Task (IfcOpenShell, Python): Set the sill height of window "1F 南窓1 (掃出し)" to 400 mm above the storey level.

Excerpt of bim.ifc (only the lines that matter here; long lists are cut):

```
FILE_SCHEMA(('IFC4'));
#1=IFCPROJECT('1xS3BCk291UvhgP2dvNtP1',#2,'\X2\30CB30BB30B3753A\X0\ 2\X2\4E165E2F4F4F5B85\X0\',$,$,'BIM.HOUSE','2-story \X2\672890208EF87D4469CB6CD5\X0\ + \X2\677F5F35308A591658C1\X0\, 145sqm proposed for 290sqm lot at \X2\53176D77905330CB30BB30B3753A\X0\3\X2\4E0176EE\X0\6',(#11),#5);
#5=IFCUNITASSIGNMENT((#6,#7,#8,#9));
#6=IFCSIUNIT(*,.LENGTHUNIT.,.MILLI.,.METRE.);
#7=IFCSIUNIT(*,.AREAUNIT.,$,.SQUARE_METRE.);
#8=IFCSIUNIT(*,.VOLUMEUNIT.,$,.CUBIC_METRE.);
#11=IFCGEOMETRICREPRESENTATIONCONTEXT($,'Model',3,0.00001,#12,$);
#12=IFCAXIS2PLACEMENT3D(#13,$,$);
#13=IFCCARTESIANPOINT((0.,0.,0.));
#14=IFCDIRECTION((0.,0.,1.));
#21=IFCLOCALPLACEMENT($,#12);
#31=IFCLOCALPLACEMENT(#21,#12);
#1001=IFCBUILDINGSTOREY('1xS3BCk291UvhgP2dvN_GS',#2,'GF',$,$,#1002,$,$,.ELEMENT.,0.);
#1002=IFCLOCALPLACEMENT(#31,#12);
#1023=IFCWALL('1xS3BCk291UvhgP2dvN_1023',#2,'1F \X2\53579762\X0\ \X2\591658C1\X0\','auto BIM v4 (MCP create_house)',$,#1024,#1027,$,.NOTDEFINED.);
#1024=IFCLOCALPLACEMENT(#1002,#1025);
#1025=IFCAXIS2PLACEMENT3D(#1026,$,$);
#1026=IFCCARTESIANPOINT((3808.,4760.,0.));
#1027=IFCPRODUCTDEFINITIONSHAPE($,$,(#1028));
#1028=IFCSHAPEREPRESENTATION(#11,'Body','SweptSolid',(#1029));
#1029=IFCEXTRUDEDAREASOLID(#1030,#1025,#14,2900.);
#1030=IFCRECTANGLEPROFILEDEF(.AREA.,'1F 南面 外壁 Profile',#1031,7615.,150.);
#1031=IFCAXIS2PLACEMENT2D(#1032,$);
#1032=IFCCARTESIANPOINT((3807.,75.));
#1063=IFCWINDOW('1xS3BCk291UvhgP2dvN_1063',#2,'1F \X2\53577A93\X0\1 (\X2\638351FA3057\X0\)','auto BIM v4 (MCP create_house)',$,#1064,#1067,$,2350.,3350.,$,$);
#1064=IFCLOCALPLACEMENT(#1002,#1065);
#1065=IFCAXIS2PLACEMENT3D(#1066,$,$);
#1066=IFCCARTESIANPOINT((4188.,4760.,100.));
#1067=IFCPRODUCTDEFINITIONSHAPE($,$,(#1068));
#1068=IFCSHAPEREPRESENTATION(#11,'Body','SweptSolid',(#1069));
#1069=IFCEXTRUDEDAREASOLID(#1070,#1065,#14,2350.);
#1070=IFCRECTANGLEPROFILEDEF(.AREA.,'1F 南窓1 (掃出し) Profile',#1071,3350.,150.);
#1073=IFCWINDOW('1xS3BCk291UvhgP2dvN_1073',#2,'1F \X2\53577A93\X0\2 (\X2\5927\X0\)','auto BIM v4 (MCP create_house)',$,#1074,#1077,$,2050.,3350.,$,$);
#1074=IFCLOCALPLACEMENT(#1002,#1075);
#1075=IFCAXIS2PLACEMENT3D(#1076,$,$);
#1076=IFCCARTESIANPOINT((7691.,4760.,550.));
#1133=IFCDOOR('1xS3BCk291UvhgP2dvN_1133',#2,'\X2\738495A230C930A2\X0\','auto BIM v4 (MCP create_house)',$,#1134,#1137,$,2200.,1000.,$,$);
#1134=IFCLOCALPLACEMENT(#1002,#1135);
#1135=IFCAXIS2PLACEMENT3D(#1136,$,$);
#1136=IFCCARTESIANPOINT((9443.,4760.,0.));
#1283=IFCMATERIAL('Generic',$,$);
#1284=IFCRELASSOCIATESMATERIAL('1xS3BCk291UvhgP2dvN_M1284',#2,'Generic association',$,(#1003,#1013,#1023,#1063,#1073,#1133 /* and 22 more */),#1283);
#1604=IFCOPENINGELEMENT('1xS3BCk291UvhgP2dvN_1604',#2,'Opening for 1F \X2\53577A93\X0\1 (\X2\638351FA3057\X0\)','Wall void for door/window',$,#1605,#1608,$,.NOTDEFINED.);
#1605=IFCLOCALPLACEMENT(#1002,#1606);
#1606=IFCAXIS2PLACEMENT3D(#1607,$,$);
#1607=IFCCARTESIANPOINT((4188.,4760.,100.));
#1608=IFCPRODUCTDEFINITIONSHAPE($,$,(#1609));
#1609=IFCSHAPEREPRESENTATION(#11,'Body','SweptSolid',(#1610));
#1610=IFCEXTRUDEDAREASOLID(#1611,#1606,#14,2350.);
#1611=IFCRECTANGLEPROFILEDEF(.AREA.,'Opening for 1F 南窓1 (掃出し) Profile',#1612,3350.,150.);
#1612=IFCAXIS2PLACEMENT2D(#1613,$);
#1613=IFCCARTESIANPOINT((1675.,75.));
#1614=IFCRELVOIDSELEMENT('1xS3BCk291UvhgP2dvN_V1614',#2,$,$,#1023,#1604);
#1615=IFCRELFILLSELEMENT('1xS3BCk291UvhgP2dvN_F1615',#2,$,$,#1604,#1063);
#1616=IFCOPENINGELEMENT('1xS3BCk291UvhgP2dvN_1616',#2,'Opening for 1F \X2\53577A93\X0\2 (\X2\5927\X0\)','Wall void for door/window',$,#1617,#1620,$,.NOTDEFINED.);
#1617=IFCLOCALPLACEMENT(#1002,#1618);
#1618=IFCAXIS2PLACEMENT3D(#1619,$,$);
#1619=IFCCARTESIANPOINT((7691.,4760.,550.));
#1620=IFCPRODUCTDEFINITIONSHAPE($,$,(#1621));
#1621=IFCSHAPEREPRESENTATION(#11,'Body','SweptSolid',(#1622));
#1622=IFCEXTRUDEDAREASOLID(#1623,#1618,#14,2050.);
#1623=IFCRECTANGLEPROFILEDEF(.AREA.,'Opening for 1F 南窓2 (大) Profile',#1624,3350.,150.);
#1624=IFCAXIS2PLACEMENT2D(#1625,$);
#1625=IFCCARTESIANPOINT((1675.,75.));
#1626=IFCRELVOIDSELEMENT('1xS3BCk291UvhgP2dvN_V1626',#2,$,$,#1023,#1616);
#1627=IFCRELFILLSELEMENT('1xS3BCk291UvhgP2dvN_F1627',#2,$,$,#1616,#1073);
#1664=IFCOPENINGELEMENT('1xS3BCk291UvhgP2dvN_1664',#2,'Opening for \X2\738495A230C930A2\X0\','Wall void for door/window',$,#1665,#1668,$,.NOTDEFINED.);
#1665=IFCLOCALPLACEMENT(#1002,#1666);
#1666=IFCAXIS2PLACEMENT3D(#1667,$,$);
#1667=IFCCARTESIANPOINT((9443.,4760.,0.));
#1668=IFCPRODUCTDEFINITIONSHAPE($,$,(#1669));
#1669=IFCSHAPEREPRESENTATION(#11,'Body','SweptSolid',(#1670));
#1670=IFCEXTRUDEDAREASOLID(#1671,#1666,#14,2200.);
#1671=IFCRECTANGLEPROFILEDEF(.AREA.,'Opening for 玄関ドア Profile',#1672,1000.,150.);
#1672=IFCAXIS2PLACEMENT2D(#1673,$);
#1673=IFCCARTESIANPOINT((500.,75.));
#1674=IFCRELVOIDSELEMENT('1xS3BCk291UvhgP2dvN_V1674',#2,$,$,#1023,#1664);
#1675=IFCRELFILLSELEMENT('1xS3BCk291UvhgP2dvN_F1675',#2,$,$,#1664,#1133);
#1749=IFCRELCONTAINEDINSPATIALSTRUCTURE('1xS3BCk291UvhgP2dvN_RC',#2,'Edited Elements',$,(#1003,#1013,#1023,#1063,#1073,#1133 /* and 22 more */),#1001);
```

```python
import numpy as np
import ifcopenshell
import ifcopenshell.api.geometry
import ifcopenshell.geom
import ifcopenshell.util.element
import ifcopenshell.util.placement
import ifcopenshell.util.shape
import ifcopenshell.util.unit

model = ifcopenshell.open("bim.ifc")
unit_scale = ifcopenshell.util.unit.calculate_unit_scale(model)

window = model.by_guid("1xS3BCk291UvhgP2dvN_1063")
opening = window.FillsVoids[0].RelatingOpeningElement
storey = ifcopenshell.util.element.get_container(window, ifc_class="IfcBuildingStorey")
level = ifcopenshell.util.placement.get_local_placement(storey.ObjectPlacement)[2, 3]

# The opening's origin need not be at the sill, so measure its lowest point.
shape = ifcopenshell.geom.create_shape(ifcopenshell.geom.settings(), opening)
bottom = ifcopenshell.util.shape.get_shape_bottom_elevation(shape, shape.geometry) / unit_scale
dz = level + 0.4 / unit_scale - bottom

shift = np.array([0.0, 0.0, dz])
# The window is not placed relative to its opening, so move both.
for product in (opening, window):
    matrix = ifcopenshell.util.placement.get_local_placement(product.ObjectPlacement)
    matrix[:3, 3] += shift
    ifcopenshell.api.geometry.edit_object_placement(model, product=product, matrix=matrix, is_si=False)

print(f"moved by {dz * unit_scale:+.3f} m")

model.write("bim_rev.ifc")
```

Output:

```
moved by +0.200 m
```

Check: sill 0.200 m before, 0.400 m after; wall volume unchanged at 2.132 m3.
